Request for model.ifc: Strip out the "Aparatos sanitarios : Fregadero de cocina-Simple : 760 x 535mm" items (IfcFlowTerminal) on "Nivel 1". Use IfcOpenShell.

First a look at what the model holds.

```python
import ifcopenshell
import ifcopenshell.util.element

model = ifcopenshell.open("model.ifc")
print(model.schema)
storey = next(s for s in model.by_type("IfcBuildingStorey") if s.Name == "Nivel 1")
terminals = [e for e in ifcopenshell.util.element.get_decomposition(storey) if e.is_a("IfcFlowTerminal")]
seen = {}
for e in terminals:
    element_type = ifcopenshell.util.element.get_type(e)
    name = element_type.Name if element_type not in (None, e) else None
    seen[name] = seen.get(name, 0) + 1
for name, count in sorted(seen.items(), key=str):
    print(count, "x", name)
```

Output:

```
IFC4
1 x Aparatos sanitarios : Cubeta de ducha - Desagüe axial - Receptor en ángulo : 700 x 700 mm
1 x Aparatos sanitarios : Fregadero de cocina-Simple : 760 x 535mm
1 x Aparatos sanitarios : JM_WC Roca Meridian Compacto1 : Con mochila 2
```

```python
import ifcopenshell
import ifcopenshell.api.root
import ifcopenshell.util.element

model = ifcopenshell.open("model.ifc")

storey = next(s for s in model.by_type("IfcBuildingStorey") if s.Name == "Nivel 1")
terminals = [e for e in ifcopenshell.util.element.get_decomposition(storey) if e.is_a("IfcFlowTerminal")]
targets = [e for e in terminals if (t := ifcopenshell.util.element.get_type(e)) not in (None, e) and t.Name == "Aparatos sanitarios : Fregadero de cocina-Simple : 760 x 535mm"]

for e in targets:
    ifcopenshell.api.root.remove_product(model, product=e)
print(len(targets), "removed")

model.write("model_updated.ifc")
```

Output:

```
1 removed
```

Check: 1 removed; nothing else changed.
